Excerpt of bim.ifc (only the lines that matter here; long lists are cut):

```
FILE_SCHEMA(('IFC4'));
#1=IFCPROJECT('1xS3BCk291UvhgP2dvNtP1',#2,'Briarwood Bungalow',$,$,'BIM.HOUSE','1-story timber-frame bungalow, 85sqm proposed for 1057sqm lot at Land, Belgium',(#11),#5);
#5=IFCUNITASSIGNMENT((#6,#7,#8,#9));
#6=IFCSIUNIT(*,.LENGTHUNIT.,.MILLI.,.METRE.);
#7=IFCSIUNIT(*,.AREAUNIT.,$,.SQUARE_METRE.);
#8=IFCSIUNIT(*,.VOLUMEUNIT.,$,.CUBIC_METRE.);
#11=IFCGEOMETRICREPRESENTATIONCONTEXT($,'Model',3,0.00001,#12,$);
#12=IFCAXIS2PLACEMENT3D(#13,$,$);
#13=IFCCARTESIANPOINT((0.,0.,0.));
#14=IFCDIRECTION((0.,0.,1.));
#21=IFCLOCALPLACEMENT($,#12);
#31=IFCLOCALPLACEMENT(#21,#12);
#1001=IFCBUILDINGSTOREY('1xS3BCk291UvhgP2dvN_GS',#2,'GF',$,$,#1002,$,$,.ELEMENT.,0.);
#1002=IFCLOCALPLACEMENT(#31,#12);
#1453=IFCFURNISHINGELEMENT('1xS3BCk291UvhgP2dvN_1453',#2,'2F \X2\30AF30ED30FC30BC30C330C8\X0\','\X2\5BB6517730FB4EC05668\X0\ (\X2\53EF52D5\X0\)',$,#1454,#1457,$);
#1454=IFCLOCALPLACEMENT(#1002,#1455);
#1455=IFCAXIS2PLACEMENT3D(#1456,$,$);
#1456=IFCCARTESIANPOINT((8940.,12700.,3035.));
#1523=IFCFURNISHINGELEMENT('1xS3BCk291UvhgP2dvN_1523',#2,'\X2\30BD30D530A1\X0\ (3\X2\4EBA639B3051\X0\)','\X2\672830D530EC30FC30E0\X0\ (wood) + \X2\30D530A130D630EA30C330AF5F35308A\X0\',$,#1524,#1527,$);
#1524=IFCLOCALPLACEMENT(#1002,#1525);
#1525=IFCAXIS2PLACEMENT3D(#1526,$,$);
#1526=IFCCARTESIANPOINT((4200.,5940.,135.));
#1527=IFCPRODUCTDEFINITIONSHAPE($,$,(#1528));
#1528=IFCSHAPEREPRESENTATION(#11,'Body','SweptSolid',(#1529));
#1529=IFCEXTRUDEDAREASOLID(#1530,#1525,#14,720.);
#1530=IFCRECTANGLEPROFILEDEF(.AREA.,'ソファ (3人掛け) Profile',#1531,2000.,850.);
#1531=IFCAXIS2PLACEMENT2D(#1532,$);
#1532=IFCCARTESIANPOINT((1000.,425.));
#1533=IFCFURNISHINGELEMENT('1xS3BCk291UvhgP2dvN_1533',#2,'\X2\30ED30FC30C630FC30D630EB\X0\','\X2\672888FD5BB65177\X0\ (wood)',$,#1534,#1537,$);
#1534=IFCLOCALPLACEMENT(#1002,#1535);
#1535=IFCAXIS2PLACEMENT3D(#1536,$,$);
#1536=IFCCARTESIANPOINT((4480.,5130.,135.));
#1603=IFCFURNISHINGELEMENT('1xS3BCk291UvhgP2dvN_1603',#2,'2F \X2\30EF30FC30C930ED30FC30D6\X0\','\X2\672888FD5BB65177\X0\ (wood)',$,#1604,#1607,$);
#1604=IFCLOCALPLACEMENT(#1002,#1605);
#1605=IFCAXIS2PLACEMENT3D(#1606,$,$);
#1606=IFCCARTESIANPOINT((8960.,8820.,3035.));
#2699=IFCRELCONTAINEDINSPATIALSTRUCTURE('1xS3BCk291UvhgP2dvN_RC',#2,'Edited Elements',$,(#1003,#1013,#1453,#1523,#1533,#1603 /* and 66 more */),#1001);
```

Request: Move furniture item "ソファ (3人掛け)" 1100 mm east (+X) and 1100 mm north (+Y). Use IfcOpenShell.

```python
import ifcopenshell
import ifcopenshell.api.geometry
import ifcopenshell.util.placement

model = ifcopenshell.open("bim.ifc")

item = model.by_id(1523)
matrix = ifcopenshell.util.placement.get_local_placement(item.ObjectPlacement)
matrix[0, 3] += 1100.0
matrix[1, 3] += 1100.0
ifcopenshell.api.geometry.edit_object_placement(model, product=item, matrix=matrix, is_si=False)

print(ifcopenshell.util.placement.get_local_placement(item.ObjectPlacement).round(3) + 0.0)

model.write("bim_v2.ifc")
```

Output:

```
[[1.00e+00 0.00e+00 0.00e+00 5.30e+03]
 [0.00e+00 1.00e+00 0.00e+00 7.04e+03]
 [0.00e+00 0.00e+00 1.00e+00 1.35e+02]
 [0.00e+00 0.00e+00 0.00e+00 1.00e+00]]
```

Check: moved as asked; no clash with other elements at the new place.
